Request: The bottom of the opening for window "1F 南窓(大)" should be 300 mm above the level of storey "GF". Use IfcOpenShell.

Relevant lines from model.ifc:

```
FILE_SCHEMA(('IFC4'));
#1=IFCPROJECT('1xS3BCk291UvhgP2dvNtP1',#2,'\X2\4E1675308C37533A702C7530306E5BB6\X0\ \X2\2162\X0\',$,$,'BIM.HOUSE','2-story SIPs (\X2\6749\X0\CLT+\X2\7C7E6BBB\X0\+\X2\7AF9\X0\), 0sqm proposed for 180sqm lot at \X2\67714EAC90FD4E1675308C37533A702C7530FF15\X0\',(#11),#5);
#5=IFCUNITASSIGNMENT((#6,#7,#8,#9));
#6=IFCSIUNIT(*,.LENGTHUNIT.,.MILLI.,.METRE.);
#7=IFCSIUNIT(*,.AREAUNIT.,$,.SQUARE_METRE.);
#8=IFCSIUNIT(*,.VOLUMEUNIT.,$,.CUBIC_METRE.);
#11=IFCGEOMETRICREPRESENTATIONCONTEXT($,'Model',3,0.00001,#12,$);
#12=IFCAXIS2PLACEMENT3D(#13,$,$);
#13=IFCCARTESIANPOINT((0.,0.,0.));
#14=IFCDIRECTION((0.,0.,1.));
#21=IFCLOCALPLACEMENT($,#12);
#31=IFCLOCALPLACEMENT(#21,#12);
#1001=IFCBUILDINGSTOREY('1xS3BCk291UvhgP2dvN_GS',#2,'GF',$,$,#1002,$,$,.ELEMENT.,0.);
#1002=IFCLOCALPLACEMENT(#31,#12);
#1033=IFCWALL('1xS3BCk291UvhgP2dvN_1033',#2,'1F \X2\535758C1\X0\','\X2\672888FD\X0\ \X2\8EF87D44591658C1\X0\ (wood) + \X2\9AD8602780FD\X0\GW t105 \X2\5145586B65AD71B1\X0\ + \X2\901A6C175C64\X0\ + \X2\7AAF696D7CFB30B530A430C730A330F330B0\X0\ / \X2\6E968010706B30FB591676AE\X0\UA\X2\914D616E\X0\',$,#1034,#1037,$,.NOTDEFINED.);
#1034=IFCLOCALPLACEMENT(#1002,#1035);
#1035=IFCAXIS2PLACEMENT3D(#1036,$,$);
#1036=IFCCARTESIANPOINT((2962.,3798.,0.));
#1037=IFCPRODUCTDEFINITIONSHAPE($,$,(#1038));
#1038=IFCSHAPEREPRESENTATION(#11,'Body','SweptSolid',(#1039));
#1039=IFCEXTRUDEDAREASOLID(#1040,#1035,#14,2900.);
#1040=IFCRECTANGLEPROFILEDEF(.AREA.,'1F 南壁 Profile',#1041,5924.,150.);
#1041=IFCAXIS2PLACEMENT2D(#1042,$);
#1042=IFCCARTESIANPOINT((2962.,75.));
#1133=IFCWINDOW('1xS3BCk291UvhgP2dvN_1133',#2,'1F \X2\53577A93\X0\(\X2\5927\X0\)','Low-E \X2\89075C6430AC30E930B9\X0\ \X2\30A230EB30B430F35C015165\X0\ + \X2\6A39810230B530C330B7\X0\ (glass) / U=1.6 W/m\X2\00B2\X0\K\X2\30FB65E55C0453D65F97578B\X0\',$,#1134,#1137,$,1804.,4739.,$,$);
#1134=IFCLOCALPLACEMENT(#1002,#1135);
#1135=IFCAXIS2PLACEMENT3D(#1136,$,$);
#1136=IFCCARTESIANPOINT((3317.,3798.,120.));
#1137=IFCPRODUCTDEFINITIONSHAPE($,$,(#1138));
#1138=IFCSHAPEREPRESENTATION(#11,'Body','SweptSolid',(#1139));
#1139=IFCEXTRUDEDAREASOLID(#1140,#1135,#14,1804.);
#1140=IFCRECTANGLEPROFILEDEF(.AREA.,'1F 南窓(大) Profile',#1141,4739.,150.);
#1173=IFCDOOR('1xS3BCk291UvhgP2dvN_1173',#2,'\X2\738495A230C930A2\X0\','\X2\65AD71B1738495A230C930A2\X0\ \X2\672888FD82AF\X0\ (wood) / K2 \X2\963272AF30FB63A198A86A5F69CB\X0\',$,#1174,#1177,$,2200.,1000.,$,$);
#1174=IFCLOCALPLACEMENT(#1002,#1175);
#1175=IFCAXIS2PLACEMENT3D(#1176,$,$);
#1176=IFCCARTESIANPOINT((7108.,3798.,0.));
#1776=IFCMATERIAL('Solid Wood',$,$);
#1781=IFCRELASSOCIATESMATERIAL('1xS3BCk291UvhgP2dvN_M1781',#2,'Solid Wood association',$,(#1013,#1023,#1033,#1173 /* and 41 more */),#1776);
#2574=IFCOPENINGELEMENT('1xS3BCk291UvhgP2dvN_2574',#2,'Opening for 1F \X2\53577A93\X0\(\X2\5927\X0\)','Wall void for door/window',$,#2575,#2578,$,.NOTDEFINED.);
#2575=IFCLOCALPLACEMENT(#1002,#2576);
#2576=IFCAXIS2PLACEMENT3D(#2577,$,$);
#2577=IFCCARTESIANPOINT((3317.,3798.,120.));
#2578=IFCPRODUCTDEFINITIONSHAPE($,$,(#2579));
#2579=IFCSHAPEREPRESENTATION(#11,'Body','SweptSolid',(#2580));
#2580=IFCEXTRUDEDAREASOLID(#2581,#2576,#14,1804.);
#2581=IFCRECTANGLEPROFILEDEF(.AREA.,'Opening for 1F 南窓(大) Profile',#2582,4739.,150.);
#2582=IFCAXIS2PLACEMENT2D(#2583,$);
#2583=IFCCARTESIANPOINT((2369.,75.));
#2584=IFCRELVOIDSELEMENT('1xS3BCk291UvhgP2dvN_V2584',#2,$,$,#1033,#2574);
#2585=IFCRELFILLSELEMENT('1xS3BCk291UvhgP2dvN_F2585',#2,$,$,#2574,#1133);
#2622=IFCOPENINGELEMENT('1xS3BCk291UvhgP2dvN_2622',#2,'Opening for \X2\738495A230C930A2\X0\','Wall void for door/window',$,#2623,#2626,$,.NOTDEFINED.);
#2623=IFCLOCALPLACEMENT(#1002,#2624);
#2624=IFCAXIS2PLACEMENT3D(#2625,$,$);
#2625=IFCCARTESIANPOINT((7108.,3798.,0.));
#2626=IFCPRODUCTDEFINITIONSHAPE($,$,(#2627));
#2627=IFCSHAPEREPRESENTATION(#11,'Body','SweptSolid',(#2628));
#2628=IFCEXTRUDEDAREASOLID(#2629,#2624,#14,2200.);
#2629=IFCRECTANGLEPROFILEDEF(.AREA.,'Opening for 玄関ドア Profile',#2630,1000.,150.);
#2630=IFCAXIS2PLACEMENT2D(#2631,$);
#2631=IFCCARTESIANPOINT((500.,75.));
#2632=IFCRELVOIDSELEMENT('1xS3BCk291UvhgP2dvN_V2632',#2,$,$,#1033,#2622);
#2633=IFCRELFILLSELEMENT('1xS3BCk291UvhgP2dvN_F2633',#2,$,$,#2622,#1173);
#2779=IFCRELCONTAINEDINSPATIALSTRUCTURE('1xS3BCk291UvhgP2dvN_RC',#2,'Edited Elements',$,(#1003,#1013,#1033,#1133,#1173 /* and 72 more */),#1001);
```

```python
import numpy as np
import ifcopenshell
import ifcopenshell.api.geometry
import ifcopenshell.geom
import ifcopenshell.util.element
import ifcopenshell.util.placement
import ifcopenshell.util.shape
import ifcopenshell.util.unit

model = ifcopenshell.open("model.ifc")
unit_scale = ifcopenshell.util.unit.calculate_unit_scale(model)

window = model.by_guid("1xS3BCk291UvhgP2dvN_1133")
opening = window.FillsVoids[0].RelatingOpeningElement
storey = ifcopenshell.util.element.get_container(window, ifc_class="IfcBuildingStorey")
level = ifcopenshell.util.placement.get_local_placement(storey.ObjectPlacement)[2, 3]

# The opening's origin need not be at the sill, so measure its lowest point.
shape = ifcopenshell.geom.create_shape(ifcopenshell.geom.settings(), opening)
bottom = ifcopenshell.util.shape.get_shape_bottom_elevation(shape, shape.geometry) / unit_scale
dz = level + 300.0 - bottom

shift = np.array([0.0, 0.0, dz])
# The window is not placed relative to its opening, so move both.
for product in (opening, window):
    matrix = ifcopenshell.util.placement.get_local_placement(product.ObjectPlacement)
    matrix[:3, 3] += shift
    ifcopenshell.api.geometry.edit_object_placement(model, product=product, matrix=matrix, is_si=False)

print(f"moved by {dz * unit_scale:+.3f} m")

model.write("model_rev.ifc")
```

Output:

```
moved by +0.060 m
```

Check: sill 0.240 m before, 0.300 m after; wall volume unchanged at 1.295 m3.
